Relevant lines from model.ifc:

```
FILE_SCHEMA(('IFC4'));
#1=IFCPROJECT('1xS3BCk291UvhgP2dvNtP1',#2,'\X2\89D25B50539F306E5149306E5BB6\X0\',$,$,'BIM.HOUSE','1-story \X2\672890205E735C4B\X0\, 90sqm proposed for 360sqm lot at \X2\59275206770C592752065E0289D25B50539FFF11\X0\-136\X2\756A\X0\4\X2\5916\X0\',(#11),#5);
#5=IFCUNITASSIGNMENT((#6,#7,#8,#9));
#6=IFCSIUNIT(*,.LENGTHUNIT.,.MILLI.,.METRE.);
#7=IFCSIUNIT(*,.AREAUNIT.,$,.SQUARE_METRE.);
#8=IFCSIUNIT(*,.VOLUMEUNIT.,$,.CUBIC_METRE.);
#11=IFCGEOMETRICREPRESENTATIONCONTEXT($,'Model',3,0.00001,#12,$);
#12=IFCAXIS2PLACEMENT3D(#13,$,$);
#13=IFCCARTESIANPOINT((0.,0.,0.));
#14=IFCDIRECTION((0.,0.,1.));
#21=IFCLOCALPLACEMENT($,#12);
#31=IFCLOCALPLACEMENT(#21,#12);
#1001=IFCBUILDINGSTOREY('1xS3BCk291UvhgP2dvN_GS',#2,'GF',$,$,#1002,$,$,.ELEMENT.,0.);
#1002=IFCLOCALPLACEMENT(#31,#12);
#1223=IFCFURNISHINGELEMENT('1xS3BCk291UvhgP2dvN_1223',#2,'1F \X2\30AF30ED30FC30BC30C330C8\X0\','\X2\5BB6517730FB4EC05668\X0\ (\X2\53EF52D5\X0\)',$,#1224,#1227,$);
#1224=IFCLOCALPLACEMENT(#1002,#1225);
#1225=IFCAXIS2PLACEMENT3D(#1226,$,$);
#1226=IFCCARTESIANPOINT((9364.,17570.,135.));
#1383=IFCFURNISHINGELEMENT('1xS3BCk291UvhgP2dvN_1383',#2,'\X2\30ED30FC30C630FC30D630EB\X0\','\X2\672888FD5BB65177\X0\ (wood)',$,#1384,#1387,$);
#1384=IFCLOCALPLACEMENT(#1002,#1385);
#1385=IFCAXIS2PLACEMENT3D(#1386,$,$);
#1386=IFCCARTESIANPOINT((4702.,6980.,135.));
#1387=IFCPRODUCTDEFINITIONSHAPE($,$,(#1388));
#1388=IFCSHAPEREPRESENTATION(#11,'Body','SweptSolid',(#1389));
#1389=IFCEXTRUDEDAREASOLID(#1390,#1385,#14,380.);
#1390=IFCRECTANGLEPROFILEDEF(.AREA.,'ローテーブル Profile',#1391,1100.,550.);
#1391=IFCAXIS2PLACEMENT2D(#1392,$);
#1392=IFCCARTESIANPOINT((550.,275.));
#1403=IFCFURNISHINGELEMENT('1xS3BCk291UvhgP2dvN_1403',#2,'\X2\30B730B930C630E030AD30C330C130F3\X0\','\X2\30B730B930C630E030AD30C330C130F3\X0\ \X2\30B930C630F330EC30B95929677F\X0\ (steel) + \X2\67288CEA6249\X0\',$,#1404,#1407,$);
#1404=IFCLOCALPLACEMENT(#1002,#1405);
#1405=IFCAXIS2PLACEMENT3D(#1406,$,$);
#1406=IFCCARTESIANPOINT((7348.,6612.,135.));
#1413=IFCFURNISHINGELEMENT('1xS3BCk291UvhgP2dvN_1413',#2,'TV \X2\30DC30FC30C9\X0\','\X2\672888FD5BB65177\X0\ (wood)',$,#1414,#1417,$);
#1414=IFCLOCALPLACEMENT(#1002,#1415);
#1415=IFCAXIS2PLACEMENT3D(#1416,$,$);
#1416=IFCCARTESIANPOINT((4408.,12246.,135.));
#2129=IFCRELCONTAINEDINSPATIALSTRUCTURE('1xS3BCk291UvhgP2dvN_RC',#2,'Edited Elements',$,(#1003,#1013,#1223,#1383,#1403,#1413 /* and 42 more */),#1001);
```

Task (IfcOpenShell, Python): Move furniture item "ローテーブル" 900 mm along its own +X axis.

```python
import ifcopenshell
import ifcopenshell.api.geometry
import ifcopenshell.util.placement

model = ifcopenshell.open("model.ifc")

item = model.by_guid("1xS3BCk291UvhgP2dvN_1383")
matrix = ifcopenshell.util.placement.get_local_placement(item.ObjectPlacement)
matrix[:3, 3] += matrix[:3, 0] * 900.0
ifcopenshell.api.geometry.edit_object_placement(model, product=item, matrix=matrix, is_si=False)

print(ifcopenshell.util.placement.get_local_placement(item.ObjectPlacement).round(3) + 0.0)

model.write("model_v2.ifc")
```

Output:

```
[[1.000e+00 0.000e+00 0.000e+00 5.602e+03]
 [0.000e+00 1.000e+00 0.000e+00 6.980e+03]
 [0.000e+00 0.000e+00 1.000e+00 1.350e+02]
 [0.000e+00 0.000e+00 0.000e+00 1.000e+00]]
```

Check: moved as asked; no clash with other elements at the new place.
